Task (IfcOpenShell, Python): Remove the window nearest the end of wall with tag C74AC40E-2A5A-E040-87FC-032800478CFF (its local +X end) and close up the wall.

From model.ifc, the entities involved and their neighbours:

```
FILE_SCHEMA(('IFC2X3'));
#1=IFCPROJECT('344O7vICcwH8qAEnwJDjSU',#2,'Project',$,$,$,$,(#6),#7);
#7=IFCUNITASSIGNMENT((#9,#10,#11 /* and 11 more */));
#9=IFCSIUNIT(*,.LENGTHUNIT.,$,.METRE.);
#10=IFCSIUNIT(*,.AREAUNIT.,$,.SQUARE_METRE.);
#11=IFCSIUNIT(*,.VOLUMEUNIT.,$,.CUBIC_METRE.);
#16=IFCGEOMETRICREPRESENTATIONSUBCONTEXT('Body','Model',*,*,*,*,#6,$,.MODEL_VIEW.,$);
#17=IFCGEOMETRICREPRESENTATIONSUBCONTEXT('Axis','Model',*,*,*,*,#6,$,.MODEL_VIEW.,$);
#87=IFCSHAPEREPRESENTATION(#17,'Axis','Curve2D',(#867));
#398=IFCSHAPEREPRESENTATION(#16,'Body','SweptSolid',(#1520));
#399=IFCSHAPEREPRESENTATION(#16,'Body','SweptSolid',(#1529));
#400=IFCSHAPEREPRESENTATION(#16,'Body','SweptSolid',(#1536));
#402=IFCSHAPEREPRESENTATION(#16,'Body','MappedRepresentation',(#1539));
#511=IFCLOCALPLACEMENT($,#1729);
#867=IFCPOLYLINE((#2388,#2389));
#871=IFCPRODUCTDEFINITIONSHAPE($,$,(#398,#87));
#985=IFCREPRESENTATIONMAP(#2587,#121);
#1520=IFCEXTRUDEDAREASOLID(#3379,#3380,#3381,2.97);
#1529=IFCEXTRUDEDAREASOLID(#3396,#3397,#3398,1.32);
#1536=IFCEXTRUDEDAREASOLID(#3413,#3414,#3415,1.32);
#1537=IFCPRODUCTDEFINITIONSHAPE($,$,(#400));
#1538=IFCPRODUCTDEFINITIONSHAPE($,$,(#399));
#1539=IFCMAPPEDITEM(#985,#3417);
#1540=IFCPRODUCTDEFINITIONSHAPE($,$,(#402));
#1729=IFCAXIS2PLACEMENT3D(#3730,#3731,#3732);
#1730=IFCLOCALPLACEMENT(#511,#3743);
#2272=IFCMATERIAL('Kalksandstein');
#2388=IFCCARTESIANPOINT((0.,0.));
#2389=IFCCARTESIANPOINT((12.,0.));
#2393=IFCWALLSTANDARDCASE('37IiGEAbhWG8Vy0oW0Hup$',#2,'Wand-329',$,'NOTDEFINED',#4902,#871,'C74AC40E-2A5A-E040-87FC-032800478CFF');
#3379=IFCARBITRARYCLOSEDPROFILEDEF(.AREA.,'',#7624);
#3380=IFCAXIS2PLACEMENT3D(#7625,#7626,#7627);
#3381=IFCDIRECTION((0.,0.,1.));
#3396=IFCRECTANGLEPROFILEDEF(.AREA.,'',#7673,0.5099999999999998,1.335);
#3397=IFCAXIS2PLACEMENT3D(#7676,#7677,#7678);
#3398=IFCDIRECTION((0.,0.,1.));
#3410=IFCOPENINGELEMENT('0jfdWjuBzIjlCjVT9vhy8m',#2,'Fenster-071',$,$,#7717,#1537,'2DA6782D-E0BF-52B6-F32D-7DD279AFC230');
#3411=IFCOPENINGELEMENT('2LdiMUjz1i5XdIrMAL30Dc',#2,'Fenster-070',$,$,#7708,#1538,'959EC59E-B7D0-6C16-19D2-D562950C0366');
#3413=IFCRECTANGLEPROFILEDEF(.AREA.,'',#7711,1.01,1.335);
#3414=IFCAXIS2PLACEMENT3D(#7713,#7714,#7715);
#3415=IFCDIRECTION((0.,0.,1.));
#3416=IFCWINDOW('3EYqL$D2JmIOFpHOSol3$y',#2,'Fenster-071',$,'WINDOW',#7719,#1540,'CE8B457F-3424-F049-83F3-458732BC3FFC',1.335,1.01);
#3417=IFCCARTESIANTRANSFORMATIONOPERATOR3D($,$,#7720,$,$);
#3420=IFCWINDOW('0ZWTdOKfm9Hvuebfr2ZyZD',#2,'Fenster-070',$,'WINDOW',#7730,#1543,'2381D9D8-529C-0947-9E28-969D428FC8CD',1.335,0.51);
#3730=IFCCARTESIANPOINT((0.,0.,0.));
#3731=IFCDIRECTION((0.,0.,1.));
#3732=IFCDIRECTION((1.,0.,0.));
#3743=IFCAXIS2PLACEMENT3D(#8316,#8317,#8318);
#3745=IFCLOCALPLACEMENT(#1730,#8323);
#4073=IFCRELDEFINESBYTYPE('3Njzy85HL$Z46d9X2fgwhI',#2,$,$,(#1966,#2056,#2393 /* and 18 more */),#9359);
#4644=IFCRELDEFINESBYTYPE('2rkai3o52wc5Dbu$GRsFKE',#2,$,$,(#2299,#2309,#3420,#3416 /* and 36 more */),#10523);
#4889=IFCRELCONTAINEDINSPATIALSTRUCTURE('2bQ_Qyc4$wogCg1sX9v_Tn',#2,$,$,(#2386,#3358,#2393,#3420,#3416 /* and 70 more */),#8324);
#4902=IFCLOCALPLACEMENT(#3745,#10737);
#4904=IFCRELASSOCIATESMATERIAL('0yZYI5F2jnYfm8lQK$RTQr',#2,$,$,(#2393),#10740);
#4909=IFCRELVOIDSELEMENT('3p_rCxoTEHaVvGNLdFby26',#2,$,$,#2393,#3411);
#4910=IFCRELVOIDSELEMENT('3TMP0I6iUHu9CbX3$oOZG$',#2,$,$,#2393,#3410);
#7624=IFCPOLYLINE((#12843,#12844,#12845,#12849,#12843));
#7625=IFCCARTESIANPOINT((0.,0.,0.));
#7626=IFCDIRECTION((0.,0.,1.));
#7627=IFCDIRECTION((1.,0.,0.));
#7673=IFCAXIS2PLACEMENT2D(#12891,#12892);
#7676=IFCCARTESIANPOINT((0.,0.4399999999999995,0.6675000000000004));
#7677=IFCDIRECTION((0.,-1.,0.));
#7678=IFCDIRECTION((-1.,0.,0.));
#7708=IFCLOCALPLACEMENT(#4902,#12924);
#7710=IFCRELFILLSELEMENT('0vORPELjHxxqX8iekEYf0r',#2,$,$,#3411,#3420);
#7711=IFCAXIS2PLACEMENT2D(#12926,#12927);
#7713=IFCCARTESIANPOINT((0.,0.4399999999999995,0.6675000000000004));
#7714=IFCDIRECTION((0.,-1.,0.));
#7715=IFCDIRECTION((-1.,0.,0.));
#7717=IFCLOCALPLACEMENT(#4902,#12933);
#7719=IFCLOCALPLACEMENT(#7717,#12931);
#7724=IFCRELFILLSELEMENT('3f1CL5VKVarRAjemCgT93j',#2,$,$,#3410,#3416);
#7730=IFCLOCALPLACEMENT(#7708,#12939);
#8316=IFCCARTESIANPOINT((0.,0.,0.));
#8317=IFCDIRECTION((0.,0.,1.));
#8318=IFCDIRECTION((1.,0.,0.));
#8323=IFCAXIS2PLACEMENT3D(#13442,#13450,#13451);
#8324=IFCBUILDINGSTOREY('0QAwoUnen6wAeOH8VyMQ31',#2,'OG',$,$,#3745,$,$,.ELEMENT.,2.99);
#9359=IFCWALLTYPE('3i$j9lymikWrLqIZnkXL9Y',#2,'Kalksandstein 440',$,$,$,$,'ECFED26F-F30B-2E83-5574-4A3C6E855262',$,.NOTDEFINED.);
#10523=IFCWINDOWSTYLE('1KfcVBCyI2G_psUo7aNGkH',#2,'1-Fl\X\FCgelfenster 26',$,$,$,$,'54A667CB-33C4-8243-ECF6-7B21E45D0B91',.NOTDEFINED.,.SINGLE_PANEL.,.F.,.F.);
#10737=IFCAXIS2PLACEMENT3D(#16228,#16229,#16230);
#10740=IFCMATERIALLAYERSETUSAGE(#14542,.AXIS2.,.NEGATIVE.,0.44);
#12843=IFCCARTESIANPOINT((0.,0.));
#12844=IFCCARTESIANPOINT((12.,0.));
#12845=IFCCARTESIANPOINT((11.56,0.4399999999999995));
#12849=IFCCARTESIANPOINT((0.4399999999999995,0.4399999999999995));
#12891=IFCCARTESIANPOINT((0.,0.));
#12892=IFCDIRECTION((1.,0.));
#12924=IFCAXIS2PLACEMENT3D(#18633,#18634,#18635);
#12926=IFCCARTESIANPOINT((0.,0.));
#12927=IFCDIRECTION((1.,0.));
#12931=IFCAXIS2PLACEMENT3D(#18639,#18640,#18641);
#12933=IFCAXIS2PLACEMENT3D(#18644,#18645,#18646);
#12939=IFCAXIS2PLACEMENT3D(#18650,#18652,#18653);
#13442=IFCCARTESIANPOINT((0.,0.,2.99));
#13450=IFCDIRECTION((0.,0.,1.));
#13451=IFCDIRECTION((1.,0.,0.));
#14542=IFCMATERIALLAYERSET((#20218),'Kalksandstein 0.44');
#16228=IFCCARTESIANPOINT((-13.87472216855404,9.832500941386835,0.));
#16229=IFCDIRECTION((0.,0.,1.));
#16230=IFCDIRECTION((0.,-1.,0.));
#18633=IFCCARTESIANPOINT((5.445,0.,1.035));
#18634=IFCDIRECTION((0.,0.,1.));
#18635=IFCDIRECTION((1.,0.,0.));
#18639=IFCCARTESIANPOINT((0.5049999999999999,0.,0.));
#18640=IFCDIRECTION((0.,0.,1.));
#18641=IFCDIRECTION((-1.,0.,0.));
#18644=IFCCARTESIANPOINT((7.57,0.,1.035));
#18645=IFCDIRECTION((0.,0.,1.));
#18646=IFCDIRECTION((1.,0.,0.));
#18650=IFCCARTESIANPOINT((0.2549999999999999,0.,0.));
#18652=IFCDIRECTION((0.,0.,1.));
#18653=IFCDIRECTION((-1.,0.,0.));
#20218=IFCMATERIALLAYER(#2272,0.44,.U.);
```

```python
import ifcopenshell
import ifcopenshell.api.feature
import ifcopenshell.api.root
import ifcopenshell.geom
import ifcopenshell.util.shape

model = ifcopenshell.open("model.ifc")
settings = ifcopenshell.geom.settings()


def volume(element):
    """Net volume in cubic metres, openings subtracted."""
    shape = ifcopenshell.geom.create_shape(settings, element)
    return ifcopenshell.util.shape.get_volume(shape.geometry)


window = model.by_guid("3EYqL$D2JmIOFpHOSol3$y")
opening = window.FillsVoids[0].RelatingOpeningElement
wall = opening.VoidsElements[0].RelatingBuildingElement
before = volume(wall)

ifcopenshell.api.root.remove_product(model, product=window)
ifcopenshell.api.feature.remove_feature(model, feature=opening)

after = volume(wall)

print(f"wall volume {before:.3f} -> {after:.3f} m3")

model.write("model_rev.ifc")
```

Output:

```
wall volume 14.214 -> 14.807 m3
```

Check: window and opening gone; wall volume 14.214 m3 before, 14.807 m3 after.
